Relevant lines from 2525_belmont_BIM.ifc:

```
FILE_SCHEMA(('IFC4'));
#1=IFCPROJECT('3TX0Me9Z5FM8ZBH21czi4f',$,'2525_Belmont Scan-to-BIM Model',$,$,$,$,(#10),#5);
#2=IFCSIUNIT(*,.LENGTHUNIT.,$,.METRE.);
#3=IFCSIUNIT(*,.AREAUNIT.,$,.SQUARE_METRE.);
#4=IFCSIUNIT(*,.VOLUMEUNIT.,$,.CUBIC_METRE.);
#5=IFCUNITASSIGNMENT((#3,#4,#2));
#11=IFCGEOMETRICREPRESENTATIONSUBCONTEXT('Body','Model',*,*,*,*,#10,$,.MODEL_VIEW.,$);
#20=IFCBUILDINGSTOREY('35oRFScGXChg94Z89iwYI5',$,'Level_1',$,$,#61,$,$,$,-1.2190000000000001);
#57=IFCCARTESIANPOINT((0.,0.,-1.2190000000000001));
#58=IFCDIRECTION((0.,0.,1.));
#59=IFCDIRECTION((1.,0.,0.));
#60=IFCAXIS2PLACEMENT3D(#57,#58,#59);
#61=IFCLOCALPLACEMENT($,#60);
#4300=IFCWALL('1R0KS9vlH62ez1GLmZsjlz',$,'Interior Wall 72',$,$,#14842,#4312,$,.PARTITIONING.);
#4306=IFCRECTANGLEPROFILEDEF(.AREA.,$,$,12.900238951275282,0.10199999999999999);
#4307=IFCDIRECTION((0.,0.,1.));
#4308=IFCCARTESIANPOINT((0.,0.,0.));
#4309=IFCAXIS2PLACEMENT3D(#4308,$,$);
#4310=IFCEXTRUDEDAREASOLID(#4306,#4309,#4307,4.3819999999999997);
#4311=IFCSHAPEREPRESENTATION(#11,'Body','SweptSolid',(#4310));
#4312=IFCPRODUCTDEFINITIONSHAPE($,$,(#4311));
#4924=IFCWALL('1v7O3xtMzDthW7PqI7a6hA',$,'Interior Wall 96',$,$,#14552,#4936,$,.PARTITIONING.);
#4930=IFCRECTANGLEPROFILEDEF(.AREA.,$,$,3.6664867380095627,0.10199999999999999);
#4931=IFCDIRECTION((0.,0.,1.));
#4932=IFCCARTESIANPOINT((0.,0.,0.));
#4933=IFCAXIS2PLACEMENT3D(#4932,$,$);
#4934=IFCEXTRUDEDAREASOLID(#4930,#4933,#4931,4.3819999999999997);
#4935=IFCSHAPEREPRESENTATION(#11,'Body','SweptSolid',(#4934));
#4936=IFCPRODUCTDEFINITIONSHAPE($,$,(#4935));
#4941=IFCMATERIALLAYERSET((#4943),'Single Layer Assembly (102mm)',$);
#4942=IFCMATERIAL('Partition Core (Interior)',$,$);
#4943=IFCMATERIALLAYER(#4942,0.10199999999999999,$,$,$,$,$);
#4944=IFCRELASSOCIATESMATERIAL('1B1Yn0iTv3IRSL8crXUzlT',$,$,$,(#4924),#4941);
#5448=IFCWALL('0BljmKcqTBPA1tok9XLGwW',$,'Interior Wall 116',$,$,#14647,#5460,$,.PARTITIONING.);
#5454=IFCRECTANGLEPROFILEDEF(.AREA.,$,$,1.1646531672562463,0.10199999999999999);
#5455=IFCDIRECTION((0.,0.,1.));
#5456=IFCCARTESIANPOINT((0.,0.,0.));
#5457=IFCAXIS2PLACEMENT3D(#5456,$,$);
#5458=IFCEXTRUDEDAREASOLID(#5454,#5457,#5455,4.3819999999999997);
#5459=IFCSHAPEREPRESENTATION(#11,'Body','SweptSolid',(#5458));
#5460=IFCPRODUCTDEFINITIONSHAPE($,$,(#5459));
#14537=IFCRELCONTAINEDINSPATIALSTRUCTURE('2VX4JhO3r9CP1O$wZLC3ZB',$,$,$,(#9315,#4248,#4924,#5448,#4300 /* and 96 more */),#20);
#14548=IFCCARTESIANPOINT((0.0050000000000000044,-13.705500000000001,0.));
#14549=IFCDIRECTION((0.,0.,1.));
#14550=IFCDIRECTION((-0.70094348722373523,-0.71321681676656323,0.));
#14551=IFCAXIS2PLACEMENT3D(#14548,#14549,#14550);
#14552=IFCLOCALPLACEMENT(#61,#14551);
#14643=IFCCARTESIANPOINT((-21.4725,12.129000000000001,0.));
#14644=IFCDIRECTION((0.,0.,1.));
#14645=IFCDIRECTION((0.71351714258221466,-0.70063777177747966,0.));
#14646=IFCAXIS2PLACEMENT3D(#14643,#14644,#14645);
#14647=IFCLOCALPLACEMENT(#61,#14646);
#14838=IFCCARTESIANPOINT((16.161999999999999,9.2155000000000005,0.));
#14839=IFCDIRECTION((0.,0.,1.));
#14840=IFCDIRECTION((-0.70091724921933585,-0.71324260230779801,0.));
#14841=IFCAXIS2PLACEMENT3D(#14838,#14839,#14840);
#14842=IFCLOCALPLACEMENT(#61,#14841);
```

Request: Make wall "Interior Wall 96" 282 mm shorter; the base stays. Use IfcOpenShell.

```python
import ifcopenshell
import ifcopenshell.geom
import ifcopenshell.util.representation
import ifcopenshell.util.shape
import ifcopenshell.util.unit

model = ifcopenshell.open("2525_belmont_BIM.ifc")
unit_scale = ifcopenshell.util.unit.calculate_unit_scale(model)
settings = ifcopenshell.geom.settings()


def volume(element):
    """Net volume in cubic metres, openings subtracted."""
    shape = ifcopenshell.geom.create_shape(settings, element)
    return ifcopenshell.util.shape.get_volume(shape.geometry)


wall = model.by_id(4924)
before = volume(wall)

body = ifcopenshell.util.representation.get_representation(wall, "Model", "Body")
solid = body.Items[0]
old_height = solid.Depth
solid.Depth -= 0.282 / unit_scale
after = volume(wall)

print(f"height {old_height:g} -> {solid.Depth:g}, volume {before:.3f} -> {after:.3f} m3")

model.write("2525_belmont_BIM_edited.ifc")
```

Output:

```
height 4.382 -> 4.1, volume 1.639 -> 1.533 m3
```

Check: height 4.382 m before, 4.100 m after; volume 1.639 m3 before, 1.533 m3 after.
